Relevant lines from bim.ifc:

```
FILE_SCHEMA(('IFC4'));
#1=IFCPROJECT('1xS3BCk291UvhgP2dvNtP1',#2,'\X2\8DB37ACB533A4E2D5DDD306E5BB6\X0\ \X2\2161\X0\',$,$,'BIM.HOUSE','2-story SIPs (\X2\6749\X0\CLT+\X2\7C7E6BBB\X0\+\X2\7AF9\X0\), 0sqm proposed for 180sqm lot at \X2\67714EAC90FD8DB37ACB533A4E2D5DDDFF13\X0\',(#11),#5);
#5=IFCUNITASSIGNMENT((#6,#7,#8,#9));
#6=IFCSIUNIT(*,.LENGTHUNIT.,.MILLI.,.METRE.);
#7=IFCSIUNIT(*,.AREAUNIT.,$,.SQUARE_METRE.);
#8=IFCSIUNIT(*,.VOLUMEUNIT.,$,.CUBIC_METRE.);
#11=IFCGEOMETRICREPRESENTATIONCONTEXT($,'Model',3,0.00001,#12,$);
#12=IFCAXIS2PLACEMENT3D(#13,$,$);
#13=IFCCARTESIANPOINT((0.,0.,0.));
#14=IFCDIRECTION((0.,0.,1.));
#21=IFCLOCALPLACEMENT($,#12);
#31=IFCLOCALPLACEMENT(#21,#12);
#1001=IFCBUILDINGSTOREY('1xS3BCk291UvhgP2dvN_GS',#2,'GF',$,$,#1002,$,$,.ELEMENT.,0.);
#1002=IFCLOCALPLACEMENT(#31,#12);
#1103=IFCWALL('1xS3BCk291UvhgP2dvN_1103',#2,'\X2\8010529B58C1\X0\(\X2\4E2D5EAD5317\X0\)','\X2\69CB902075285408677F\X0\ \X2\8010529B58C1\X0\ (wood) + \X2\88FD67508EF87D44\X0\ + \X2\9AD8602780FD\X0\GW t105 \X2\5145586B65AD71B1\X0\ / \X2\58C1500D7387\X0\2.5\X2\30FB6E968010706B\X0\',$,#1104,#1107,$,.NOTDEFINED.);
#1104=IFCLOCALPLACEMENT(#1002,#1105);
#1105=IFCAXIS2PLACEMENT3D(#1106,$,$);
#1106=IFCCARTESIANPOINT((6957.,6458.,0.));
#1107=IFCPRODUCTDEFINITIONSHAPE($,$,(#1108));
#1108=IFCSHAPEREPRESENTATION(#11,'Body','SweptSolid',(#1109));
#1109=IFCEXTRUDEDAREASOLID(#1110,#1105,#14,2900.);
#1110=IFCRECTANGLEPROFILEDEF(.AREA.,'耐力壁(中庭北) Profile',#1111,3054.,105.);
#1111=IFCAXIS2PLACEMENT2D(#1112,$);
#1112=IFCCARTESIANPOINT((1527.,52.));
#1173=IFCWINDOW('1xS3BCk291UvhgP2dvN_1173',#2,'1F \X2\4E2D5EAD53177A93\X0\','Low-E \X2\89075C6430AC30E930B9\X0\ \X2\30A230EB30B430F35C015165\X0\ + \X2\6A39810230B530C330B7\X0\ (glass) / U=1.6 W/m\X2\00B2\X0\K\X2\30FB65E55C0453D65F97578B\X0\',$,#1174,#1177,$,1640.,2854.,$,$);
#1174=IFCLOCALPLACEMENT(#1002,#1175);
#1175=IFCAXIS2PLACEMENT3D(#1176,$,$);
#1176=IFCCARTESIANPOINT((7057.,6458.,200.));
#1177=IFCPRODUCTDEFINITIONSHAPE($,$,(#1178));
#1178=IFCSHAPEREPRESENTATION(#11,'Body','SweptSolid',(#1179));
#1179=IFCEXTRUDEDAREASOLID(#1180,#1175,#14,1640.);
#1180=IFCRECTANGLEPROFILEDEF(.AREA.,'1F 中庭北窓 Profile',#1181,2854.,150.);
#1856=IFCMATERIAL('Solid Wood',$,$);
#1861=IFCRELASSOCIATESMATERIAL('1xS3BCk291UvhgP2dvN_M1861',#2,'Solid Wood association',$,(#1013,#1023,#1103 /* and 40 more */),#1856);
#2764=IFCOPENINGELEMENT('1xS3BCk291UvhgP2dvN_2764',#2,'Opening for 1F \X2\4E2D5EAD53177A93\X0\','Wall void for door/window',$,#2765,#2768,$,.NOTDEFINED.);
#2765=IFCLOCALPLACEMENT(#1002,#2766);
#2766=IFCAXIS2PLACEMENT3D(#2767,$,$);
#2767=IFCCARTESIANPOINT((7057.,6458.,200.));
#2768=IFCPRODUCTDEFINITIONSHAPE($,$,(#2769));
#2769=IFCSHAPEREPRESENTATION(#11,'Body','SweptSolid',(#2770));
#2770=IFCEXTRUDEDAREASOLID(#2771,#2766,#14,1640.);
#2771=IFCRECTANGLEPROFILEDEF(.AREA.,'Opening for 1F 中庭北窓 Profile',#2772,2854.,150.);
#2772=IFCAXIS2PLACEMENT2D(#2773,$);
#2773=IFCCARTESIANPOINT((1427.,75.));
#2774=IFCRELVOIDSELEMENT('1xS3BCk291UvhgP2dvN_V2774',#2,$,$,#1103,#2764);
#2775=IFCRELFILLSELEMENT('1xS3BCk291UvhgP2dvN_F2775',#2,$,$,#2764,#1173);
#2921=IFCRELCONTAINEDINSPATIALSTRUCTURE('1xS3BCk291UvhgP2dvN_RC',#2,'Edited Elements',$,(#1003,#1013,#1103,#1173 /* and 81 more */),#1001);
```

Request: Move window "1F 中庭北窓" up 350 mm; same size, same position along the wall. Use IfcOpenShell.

```python
import numpy as np
import ifcopenshell
import ifcopenshell.api.geometry
import ifcopenshell.util.placement
import ifcopenshell.util.unit

model = ifcopenshell.open("bim.ifc")
unit_scale = ifcopenshell.util.unit.calculate_unit_scale(model)

window = model.by_guid("1xS3BCk291UvhgP2dvN_1173")
opening = window.FillsVoids[0].RelatingOpeningElement
dz = 350.0

shift = np.array([0.0, 0.0, dz])
# The window is not placed relative to its opening, so move both.
for product in (opening, window):
    matrix = ifcopenshell.util.placement.get_local_placement(product.ObjectPlacement)
    matrix[:3, 3] += shift
    ifcopenshell.api.geometry.edit_object_placement(model, product=product, matrix=matrix, is_si=False)

print(f"moved by {dz * unit_scale:+.3f} m")

model.write("bim_rev.ifc")
```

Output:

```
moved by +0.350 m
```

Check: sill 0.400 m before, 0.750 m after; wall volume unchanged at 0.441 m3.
